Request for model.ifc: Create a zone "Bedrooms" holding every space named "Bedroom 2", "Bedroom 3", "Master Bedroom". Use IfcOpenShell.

First a look at what the model holds.

```python
import ifcopenshell

model = ifcopenshell.open("model.ifc")
print(model.schema)
seen = {}
for space in model.by_type("IfcSpace"):
    seen[space.LongName] = seen.get(space.LongName, 0) + 1
for name, count in sorted(seen.items(), key=str):
    print(count, "x", name)
print("zones:", [z.Name for z in model.by_type("IfcZone")][:20])
```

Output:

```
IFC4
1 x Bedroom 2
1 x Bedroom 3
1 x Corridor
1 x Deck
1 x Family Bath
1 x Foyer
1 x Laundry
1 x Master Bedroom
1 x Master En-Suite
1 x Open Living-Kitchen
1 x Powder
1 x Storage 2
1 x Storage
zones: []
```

```python
import ifcopenshell
import ifcopenshell.api.group
import ifcopenshell.api.root

model = ifcopenshell.open("model.ifc")

names = {"Bedroom 2", "Bedroom 3", "Master Bedroom"}
spaces = [s for s in model.by_type("IfcSpace") if s.LongName in names]

zone = ifcopenshell.api.root.create_entity(model, ifc_class="IfcZone", name="Bedrooms")
ifcopenshell.api.group.assign_group(model, products=spaces, group=zone)
print(len(spaces), "spaces in", zone.Name)

model.write("model-out.ifc")
```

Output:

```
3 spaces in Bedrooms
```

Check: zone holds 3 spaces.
